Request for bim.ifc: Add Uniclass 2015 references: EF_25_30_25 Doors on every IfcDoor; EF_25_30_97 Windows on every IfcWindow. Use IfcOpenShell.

First a look at what the model holds.

```python
import ifcopenshell

model = ifcopenshell.open("bim.ifc")
print(model.schema)
print("classifications:", [c.Name for c in model.by_type("IfcClassification")])
for ifc_class in ("IfcDoor", "IfcRoof", "IfcStair", "IfcWall", "IfcWindow"):
    print(ifc_class, len(model.by_type(ifc_class)))
```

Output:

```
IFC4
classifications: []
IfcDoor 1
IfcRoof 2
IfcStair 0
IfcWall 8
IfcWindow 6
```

```python
import ifcopenshell
import ifcopenshell.api.classification

model = ifcopenshell.open("bim.ifc")

system = ifcopenshell.api.classification.add_classification(model, classification="Uniclass 2015")

codes = {
    "IfcDoor": ("EF_25_30_25", "Doors"),
    "IfcWindow": ("EF_25_30_97", "Windows"),
}
for ifc_class, (code, name) in codes.items():
    products = model.by_type(ifc_class)
    ifcopenshell.api.classification.add_reference(
        model, products=products, classification=system, identification=code, name=name
    )
    print(code, len(products))

model.write("bim_edited.ifc")
```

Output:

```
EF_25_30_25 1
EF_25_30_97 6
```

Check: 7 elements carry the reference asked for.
